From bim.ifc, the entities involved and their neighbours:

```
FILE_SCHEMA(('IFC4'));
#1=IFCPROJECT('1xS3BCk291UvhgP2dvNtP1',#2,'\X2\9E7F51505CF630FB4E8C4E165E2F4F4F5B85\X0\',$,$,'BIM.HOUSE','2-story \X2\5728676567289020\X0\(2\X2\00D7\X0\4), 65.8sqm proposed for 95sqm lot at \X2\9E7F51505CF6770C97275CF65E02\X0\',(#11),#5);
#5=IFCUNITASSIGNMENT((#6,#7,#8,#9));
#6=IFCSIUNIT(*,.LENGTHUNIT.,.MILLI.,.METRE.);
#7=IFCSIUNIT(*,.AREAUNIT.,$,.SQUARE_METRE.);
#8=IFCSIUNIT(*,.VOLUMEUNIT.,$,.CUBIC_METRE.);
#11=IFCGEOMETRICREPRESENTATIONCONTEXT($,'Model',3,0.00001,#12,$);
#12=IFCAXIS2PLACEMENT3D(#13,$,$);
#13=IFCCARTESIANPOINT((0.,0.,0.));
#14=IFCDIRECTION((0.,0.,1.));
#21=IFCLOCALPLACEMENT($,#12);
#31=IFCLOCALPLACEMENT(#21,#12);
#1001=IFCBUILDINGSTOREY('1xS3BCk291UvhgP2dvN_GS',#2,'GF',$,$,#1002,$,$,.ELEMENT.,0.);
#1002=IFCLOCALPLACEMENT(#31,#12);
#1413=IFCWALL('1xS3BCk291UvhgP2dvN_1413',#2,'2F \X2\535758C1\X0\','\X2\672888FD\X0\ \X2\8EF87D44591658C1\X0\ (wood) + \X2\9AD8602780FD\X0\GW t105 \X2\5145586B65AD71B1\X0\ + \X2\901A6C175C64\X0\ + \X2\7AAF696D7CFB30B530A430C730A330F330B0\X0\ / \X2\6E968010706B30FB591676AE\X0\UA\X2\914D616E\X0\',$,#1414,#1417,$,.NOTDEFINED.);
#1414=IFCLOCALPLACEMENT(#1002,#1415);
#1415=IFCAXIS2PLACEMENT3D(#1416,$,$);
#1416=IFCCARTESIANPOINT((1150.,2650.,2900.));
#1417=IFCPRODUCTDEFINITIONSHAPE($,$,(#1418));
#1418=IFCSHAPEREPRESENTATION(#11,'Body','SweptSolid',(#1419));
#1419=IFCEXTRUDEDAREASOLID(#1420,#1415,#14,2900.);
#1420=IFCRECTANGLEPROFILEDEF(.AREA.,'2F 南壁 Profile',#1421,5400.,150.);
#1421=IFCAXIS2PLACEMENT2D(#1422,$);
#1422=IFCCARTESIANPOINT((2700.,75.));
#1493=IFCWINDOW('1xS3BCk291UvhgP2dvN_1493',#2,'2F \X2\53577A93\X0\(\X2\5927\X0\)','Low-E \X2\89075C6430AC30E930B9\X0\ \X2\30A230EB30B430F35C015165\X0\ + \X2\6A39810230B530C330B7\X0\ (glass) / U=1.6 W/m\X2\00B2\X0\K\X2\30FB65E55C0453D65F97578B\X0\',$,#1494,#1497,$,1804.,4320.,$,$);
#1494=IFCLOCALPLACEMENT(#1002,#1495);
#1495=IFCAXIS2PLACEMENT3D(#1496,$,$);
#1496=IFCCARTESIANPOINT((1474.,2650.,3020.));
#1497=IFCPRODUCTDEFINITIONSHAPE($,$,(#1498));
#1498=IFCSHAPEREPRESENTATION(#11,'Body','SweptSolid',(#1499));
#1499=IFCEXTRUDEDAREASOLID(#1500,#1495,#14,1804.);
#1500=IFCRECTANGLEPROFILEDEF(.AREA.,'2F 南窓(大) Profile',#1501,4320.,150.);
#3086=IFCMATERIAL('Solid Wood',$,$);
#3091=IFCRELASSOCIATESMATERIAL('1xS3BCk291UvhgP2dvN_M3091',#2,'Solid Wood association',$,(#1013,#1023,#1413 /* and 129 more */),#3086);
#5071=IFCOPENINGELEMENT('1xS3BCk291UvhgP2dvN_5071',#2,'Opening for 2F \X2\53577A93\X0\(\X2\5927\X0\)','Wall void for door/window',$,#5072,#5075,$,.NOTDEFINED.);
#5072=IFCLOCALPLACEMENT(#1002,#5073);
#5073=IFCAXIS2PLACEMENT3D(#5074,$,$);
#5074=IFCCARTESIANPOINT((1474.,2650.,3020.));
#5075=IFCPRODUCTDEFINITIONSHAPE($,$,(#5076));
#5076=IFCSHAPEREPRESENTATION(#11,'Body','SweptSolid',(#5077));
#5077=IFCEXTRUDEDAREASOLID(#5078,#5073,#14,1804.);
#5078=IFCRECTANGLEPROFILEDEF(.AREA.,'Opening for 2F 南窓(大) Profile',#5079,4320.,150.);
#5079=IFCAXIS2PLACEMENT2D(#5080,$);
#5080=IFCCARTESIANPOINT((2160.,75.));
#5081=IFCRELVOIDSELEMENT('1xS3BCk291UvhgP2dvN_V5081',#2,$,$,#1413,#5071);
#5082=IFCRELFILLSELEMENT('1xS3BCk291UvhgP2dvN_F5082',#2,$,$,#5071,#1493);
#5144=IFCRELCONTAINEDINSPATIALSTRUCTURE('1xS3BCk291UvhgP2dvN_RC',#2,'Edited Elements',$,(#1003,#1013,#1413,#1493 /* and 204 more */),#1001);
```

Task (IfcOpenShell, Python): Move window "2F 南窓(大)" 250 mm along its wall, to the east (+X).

```python
import ifcopenshell
import ifcopenshell.api.geometry
import ifcopenshell.util.placement

model = ifcopenshell.open("bim.ifc")

window = model.by_id(1493)
opening = window.FillsVoids[0].RelatingOpeningElement
wall = opening.VoidsElements[0].RelatingBuildingElement

wall_matrix = ifcopenshell.util.placement.get_local_placement(wall.ObjectPlacement)
shift = wall_matrix[:3, 0] * 250.0
before = ifcopenshell.util.placement.get_local_placement(window.ObjectPlacement)[:3, 3].copy()

# The window is not placed relative to its opening, so move both.
for product in (opening, window):
    matrix = ifcopenshell.util.placement.get_local_placement(product.ObjectPlacement)
    matrix[:3, 3] += shift
    ifcopenshell.api.geometry.edit_object_placement(model, product=product, matrix=matrix, is_si=False)

after = ifcopenshell.util.placement.get_local_placement(window.ObjectPlacement)[:3, 3]
print("window moved by", (after - before).round(3) + 0.0)

model.write("bim-out.ifc")
```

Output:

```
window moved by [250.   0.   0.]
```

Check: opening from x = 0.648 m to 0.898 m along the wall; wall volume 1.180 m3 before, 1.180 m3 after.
